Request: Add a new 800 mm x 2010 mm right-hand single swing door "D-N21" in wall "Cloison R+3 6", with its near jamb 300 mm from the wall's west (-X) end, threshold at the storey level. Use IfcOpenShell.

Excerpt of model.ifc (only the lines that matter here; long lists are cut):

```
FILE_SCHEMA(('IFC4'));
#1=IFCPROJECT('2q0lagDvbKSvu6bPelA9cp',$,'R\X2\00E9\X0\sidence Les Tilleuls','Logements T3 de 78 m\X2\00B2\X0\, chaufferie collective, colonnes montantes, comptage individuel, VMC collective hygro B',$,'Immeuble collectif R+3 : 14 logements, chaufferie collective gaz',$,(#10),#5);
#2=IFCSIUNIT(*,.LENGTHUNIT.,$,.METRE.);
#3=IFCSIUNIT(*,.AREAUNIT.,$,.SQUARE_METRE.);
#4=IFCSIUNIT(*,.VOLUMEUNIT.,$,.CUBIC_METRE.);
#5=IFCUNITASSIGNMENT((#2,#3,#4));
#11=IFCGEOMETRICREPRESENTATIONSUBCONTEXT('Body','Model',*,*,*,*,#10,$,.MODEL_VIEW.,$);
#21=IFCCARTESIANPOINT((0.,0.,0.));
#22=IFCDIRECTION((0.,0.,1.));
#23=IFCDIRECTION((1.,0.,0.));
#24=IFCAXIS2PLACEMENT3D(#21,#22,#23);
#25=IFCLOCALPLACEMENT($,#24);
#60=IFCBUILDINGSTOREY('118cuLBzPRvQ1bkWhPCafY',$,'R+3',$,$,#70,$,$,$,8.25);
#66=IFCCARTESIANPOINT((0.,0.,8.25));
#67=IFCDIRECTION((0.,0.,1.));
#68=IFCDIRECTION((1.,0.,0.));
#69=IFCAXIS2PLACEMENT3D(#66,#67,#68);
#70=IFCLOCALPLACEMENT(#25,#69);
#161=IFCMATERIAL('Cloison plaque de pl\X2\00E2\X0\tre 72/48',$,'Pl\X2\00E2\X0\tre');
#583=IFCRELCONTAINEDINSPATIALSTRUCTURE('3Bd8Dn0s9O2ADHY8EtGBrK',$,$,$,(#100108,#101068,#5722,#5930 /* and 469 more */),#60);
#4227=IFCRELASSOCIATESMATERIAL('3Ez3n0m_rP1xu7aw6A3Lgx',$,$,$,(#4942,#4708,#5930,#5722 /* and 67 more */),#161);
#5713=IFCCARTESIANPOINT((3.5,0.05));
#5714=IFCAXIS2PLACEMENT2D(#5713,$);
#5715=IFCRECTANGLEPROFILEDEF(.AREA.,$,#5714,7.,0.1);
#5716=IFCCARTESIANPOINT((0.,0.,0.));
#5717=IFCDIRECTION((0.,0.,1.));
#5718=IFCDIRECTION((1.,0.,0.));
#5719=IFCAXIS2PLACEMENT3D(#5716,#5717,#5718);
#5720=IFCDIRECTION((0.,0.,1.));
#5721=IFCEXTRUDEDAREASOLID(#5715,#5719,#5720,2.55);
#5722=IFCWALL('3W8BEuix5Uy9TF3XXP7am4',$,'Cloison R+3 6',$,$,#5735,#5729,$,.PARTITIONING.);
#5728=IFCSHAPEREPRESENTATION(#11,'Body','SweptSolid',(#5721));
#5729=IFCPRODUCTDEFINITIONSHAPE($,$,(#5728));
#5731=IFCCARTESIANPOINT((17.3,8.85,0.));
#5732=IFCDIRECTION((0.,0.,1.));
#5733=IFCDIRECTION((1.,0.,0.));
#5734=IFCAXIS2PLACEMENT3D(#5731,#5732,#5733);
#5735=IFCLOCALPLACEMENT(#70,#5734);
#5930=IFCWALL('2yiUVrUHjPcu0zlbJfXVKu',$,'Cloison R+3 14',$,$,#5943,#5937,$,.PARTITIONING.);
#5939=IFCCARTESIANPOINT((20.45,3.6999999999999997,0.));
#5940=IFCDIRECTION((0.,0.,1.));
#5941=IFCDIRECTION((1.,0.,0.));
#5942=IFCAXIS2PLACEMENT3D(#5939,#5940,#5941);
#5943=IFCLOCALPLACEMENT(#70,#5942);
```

```python
import numpy as np
import ifcopenshell
import ifcopenshell.api.feature
import ifcopenshell.api.geometry
import ifcopenshell.api.root
import ifcopenshell.api.spatial
import ifcopenshell.geom
import ifcopenshell.util.element
import ifcopenshell.util.placement
import ifcopenshell.util.representation
import ifcopenshell.util.shape
import ifcopenshell.util.unit

model = ifcopenshell.open("model.ifc")
unit_scale = ifcopenshell.util.unit.calculate_unit_scale(model)
settings = ifcopenshell.geom.settings()


def volume(element):
    """Net volume in cubic metres, openings subtracted."""
    shape = ifcopenshell.geom.create_shape(settings, element)
    return ifcopenshell.util.shape.get_volume(shape.geometry)


wall = model.by_id(5722)
storey = ifcopenshell.util.element.get_container(wall, ifc_class="IfcBuildingStorey")
context = ifcopenshell.util.representation.get_context(model, "Model", "Body", "MODEL_VIEW")
before = volume(wall)

width, height, from_end, sill = 0.8, 2.01, 0.3, 0.0  # metres

# The wall runs along its own X axis, and the end named is its -X end.
wall_shape = ifcopenshell.geom.create_shape(settings, wall)
x, y, z = ifcopenshell.util.shape.get_vertices(wall_shape.geometry).T
start = x.min() + from_end
face, thickness = float(y.min()), float(y.max() - y.min())
wall_matrix = ifcopenshell.util.placement.get_local_placement(wall.ObjectPlacement)
level = ifcopenshell.util.placement.get_local_placement(storey.ObjectPlacement)[2, 3]


def in_wall(x, y):
    """Placement at x, y metres in the wall's axes, at sill height."""
    matrix = wall_matrix.copy()
    matrix[:, 3] = wall_matrix @ np.array([x / unit_scale, y / unit_scale, 0.0, 1.0])
    matrix[2, 3] = level + sill / unit_scale
    return matrix


# Opening: a box that overshoots both wall faces by 50 mm.
opening = ifcopenshell.api.root.create_entity(model, ifc_class="IfcOpeningElement", predefined_type="OPENING")
box = ifcopenshell.api.geometry.add_wall_representation(
    model, context=context, length=width, height=height, thickness=thickness + 0.1
)
ifcopenshell.api.geometry.assign_representation(model, product=opening, representation=box)
ifcopenshell.api.geometry.edit_object_placement(model, product=opening, matrix=in_wall(start, face - 0.05), is_si=False)
ifcopenshell.api.feature.add_feature(model, feature=opening, element=wall)

door = ifcopenshell.api.root.create_entity(model, ifc_class="IfcDoor", name="D-N21", predefined_type="DOOR")
door.OverallWidth, door.OverallHeight = width / unit_scale, height / unit_scale
door.OperationType = "SINGLE_SWING_RIGHT"
body = ifcopenshell.api.geometry.add_door_representation(
    model,
    context=context,
    overall_width=door.OverallWidth,
    overall_height=door.OverallHeight,
    operation_type="SINGLE_SWING_RIGHT",
    lining_properties={"LiningDepth": thickness / unit_scale, "ThresholdDepth": thickness / unit_scale},
)
ifcopenshell.api.geometry.assign_representation(model, product=door, representation=body)
ifcopenshell.api.spatial.assign_container(model, products=[door], relating_structure=storey)
ifcopenshell.api.feature.add_filling(model, opening=opening, element=door)

# The lining spans the wall, so the door starts at the wall face.
ifcopenshell.api.geometry.edit_object_placement(model, product=door, matrix=in_wall(start, face), is_si=False)

after = volume(wall)

print(f"wall volume {before:.3f} -> {after:.3f} m3")

model.write("model_rev.ifc")
```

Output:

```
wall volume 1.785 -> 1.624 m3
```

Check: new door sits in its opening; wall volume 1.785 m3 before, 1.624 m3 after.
